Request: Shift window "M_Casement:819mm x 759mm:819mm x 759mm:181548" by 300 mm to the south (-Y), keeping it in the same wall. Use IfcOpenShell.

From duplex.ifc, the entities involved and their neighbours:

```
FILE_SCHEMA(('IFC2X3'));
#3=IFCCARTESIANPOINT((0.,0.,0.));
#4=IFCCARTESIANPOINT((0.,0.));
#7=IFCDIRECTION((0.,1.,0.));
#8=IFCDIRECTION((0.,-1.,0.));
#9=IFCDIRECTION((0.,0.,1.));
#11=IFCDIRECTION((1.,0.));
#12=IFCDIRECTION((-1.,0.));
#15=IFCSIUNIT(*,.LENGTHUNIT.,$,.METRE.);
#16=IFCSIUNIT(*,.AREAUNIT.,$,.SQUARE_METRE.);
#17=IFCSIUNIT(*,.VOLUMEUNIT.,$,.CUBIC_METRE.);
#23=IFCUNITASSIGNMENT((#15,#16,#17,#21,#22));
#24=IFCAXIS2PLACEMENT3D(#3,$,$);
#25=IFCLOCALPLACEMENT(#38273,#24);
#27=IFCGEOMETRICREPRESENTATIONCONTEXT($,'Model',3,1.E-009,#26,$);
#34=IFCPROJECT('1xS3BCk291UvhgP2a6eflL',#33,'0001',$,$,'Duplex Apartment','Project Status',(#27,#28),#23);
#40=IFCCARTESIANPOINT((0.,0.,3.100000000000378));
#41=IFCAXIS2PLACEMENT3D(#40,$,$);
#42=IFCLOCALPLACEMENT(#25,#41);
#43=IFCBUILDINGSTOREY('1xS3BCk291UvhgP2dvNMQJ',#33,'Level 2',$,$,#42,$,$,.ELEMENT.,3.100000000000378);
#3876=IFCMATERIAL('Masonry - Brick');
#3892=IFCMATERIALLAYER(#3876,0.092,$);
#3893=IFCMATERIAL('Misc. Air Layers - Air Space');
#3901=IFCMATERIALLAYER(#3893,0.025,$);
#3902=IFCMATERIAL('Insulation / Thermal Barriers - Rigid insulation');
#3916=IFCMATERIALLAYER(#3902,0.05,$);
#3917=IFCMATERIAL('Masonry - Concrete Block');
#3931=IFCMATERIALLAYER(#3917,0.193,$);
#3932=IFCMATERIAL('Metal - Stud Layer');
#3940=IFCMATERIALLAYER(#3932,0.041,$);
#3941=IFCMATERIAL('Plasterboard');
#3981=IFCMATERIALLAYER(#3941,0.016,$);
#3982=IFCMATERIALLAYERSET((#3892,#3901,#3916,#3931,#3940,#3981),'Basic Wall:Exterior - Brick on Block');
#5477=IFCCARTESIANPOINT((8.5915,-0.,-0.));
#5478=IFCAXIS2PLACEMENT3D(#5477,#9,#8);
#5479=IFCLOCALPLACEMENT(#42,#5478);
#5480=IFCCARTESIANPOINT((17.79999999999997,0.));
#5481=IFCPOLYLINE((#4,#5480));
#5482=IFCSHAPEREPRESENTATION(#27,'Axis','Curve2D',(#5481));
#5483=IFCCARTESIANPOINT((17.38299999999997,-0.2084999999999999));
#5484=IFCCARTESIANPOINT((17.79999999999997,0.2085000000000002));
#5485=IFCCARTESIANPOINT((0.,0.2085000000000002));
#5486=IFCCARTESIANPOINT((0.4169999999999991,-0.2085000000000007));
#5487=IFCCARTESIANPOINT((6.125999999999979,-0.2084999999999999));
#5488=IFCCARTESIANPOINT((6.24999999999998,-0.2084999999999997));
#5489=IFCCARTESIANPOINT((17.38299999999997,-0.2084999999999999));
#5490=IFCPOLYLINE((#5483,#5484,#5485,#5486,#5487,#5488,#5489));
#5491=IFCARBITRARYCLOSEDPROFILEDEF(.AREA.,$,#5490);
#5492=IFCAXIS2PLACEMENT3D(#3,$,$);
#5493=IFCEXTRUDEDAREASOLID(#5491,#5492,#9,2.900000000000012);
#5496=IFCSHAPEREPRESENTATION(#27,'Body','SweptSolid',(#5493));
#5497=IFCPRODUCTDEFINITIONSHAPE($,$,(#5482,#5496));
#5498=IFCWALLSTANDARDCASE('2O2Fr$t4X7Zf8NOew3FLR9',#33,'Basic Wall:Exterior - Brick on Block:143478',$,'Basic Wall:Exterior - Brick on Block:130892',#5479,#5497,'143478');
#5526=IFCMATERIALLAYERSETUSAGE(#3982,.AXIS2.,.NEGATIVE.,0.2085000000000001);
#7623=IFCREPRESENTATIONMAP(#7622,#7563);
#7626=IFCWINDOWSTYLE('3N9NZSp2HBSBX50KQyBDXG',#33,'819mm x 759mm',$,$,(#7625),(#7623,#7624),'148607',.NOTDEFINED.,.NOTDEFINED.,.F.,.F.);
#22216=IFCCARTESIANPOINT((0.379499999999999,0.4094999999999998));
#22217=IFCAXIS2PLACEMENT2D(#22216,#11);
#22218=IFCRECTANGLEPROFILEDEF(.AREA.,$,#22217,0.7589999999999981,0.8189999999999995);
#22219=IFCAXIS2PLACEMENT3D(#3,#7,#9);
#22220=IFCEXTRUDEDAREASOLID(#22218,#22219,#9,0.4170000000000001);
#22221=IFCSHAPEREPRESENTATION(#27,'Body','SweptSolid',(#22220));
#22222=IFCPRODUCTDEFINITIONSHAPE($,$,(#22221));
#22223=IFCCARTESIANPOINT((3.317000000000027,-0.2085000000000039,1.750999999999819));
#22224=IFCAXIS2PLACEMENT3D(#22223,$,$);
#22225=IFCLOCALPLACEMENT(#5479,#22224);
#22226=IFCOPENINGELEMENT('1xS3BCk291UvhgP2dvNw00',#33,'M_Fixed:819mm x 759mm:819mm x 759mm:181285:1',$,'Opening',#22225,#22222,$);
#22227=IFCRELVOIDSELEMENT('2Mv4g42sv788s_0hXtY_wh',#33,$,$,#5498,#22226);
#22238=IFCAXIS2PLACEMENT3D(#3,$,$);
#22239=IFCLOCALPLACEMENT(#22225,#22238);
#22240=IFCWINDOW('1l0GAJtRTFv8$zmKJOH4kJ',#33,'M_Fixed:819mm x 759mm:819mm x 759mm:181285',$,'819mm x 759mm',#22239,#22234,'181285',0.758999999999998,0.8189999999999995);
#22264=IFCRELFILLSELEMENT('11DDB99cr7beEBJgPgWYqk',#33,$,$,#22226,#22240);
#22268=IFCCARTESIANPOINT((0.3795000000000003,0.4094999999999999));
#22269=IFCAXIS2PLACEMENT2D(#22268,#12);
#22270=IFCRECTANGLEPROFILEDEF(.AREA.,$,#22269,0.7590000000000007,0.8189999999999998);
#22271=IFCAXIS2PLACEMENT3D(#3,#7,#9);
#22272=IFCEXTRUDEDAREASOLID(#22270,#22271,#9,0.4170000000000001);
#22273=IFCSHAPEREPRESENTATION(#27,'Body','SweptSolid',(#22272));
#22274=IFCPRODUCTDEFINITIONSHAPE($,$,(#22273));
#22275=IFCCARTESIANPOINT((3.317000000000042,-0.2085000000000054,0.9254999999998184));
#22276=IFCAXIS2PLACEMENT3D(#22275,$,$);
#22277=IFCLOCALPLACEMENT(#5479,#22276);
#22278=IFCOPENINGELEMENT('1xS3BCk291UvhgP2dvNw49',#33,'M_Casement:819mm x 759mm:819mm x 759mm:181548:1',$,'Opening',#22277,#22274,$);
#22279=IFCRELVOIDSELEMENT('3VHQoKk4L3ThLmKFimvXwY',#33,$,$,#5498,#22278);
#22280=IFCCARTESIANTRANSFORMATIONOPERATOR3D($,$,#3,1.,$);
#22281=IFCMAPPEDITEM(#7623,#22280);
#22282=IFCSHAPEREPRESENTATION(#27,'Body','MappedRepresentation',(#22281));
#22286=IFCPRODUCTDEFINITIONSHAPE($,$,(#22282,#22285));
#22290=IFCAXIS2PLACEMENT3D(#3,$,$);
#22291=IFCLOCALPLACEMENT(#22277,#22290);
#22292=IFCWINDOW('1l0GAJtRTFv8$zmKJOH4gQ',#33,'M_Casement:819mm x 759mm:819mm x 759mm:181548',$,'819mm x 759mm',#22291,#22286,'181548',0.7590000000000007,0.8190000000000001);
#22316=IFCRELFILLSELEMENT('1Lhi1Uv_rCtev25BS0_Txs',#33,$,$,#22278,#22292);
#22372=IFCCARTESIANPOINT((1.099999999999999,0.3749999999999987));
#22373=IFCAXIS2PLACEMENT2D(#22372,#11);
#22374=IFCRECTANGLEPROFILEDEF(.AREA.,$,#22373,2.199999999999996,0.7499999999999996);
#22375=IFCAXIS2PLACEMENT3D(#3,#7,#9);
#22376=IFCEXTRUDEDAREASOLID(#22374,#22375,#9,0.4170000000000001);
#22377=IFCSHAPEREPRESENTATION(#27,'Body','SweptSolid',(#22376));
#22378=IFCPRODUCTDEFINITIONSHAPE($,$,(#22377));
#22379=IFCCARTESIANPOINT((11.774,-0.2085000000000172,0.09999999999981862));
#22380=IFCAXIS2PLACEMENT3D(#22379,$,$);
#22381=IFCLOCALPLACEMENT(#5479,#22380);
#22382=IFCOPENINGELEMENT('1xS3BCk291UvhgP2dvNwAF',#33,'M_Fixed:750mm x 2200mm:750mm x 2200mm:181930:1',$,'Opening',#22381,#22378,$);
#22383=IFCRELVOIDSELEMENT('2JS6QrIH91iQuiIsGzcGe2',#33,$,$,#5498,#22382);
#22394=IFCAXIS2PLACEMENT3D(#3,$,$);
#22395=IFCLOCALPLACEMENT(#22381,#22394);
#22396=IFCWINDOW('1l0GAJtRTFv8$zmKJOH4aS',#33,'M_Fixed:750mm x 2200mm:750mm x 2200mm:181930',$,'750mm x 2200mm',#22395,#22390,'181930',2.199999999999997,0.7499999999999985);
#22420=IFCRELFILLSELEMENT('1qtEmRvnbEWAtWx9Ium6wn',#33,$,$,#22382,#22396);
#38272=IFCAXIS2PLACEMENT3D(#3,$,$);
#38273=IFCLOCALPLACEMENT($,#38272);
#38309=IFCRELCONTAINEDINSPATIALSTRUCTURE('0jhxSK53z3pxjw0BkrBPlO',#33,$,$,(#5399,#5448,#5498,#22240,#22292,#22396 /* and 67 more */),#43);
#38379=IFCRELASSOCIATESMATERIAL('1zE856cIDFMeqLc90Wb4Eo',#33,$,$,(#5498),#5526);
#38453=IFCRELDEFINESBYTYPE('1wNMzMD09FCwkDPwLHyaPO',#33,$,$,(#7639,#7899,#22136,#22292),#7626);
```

```python
import ifcopenshell
import ifcopenshell.api.geometry
import ifcopenshell.util.placement
import ifcopenshell.util.unit

model = ifcopenshell.open("duplex.ifc")
unit_scale = ifcopenshell.util.unit.calculate_unit_scale(model)

window = model.by_guid("1l0GAJtRTFv8$zmKJOH4gQ")
opening = window.FillsVoids[0].RelatingOpeningElement
wall = opening.VoidsElements[0].RelatingBuildingElement

wall_matrix = ifcopenshell.util.placement.get_local_placement(wall.ObjectPlacement)
shift = wall_matrix[:3, 0] * 0.3 / unit_scale
before = ifcopenshell.util.placement.get_local_placement(window.ObjectPlacement)[:3, 3].copy()

# The window is placed relative to its opening, so it follows when the opening moves.
matrix = ifcopenshell.util.placement.get_local_placement(opening.ObjectPlacement)
matrix[:3, 3] += shift
ifcopenshell.api.geometry.edit_object_placement(
    model, product=opening, matrix=matrix, is_si=False, should_transform_children=True
)

after = ifcopenshell.util.placement.get_local_placement(window.ObjectPlacement)[:3, 3]
print("window moved by", (after - before).round(3) + 0.0)

model.write("duplex_rev.ifc")
```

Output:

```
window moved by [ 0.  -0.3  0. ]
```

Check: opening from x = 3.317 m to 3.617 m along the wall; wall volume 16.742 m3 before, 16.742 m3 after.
